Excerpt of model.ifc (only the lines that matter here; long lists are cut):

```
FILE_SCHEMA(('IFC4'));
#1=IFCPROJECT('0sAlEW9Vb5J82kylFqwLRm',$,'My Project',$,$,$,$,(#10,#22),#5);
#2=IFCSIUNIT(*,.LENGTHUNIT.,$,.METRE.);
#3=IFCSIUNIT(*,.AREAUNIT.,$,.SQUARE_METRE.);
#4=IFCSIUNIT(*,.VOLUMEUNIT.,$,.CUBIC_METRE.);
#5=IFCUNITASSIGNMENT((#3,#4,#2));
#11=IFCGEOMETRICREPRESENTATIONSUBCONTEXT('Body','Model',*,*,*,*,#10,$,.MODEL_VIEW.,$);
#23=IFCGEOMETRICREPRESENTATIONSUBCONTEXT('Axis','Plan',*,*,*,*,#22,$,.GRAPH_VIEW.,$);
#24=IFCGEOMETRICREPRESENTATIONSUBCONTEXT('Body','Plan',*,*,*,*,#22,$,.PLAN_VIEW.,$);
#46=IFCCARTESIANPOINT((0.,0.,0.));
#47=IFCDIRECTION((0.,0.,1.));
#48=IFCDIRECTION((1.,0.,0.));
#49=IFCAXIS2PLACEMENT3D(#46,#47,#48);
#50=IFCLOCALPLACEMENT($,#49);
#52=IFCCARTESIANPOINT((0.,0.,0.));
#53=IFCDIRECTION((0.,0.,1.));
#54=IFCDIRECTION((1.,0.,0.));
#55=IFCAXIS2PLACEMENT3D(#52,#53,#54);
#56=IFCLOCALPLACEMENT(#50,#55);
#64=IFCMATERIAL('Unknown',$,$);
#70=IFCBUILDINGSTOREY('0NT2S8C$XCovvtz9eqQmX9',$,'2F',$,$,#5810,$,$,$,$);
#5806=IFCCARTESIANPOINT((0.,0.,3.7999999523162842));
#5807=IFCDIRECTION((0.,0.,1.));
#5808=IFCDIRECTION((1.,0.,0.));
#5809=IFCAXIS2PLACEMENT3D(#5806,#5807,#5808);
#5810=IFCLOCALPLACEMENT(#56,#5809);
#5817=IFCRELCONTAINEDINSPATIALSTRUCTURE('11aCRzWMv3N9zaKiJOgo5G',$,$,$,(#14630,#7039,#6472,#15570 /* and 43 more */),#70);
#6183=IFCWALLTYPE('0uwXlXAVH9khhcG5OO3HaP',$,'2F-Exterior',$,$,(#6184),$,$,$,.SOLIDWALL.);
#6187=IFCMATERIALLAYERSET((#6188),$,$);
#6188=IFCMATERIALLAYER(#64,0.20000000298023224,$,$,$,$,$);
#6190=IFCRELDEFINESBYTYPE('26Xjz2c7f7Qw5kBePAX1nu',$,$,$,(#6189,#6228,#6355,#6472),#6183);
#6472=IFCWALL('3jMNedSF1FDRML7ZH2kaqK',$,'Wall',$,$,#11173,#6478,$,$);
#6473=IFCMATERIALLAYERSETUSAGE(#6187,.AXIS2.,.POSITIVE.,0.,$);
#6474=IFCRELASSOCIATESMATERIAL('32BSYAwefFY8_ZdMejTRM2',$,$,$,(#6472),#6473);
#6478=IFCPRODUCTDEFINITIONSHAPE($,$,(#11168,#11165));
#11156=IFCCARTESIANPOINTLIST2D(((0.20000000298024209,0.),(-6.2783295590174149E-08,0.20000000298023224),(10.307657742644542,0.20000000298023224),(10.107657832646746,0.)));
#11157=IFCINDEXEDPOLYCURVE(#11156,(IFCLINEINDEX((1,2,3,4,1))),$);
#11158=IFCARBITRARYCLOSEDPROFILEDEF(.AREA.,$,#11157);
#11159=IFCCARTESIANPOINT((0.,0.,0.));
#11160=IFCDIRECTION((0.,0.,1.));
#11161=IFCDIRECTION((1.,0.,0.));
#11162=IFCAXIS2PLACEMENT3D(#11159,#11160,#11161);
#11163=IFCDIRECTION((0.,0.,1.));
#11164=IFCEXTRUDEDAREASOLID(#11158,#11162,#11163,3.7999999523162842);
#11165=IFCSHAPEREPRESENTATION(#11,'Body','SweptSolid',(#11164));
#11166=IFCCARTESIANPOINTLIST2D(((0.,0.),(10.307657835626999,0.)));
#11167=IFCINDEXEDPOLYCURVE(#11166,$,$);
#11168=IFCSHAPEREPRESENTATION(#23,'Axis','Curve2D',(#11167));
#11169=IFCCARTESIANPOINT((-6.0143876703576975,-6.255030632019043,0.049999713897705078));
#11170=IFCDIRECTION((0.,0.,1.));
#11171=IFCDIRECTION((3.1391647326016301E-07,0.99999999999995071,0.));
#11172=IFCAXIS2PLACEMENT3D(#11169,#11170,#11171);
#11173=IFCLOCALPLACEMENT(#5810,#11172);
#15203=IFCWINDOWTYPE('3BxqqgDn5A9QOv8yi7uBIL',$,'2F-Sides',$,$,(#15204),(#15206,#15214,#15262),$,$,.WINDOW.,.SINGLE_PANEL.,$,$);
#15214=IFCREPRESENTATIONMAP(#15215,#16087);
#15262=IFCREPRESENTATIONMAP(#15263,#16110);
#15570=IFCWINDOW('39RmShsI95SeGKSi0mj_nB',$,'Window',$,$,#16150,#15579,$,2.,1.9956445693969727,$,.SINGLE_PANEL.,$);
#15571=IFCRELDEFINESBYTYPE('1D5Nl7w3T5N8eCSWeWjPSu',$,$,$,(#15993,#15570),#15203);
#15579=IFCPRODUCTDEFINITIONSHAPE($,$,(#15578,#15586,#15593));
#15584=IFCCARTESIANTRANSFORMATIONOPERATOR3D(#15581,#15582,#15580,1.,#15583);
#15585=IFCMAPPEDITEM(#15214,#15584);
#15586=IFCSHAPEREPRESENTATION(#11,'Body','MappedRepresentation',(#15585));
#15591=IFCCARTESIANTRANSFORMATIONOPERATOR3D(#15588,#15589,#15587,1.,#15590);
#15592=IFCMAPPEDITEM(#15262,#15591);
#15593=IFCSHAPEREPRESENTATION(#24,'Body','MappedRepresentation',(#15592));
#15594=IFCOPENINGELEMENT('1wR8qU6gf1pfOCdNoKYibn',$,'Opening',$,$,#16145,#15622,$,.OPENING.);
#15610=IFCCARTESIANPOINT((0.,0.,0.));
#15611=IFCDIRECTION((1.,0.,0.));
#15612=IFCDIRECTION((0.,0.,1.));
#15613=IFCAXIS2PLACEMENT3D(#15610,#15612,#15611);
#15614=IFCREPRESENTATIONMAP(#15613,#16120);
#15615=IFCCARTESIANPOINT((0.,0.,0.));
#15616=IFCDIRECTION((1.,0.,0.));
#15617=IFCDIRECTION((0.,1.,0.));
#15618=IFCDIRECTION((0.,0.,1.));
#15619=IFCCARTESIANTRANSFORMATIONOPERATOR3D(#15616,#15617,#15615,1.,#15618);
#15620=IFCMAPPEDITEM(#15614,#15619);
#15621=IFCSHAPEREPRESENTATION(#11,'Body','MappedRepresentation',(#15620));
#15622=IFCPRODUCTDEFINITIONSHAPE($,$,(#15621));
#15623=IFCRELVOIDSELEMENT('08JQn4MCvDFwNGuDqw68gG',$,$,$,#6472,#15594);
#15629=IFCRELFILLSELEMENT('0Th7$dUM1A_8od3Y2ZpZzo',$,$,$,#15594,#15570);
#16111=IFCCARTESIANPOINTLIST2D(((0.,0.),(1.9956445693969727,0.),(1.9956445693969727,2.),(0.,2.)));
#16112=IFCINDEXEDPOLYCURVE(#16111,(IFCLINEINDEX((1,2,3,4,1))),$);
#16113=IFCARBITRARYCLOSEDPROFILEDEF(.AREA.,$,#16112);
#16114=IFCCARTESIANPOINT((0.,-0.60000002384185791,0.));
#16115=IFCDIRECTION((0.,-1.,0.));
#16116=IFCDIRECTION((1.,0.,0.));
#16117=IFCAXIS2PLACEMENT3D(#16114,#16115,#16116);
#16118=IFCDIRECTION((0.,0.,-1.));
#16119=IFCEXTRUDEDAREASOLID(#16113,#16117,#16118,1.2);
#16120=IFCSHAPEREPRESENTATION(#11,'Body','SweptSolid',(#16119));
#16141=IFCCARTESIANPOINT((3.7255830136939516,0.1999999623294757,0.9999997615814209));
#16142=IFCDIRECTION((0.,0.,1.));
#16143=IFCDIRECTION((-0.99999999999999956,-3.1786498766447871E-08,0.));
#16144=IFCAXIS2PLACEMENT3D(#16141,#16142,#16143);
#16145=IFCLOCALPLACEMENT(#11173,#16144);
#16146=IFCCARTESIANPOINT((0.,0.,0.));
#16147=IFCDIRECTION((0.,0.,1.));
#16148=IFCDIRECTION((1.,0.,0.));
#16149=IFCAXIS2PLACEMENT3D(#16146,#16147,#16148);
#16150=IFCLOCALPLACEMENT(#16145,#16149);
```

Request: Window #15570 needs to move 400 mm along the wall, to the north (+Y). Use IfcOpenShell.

```python
import ifcopenshell
import ifcopenshell.api.geometry
import ifcopenshell.util.placement

model = ifcopenshell.open("model.ifc")

window = model.by_id(15570)
opening = window.FillsVoids[0].RelatingOpeningElement
wall = opening.VoidsElements[0].RelatingBuildingElement

wall_matrix = ifcopenshell.util.placement.get_local_placement(wall.ObjectPlacement)
shift = wall_matrix[:3, 0] * 0.4
before = ifcopenshell.util.placement.get_local_placement(window.ObjectPlacement)[:3, 3].copy()

# The window is placed relative to its opening, so it follows when the opening moves.
matrix = ifcopenshell.util.placement.get_local_placement(opening.ObjectPlacement)
matrix[:3, 3] += shift
ifcopenshell.api.geometry.edit_object_placement(
    model, product=opening, matrix=matrix, is_si=False, should_transform_children=True
)

after = ifcopenshell.util.placement.get_local_placement(window.ObjectPlacement)[:3, 3]
print("window moved by", (after - before).round(3) + 0.0)

model.write("model-out.ifc")
```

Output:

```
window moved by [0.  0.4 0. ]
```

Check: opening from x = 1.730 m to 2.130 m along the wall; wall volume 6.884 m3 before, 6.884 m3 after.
